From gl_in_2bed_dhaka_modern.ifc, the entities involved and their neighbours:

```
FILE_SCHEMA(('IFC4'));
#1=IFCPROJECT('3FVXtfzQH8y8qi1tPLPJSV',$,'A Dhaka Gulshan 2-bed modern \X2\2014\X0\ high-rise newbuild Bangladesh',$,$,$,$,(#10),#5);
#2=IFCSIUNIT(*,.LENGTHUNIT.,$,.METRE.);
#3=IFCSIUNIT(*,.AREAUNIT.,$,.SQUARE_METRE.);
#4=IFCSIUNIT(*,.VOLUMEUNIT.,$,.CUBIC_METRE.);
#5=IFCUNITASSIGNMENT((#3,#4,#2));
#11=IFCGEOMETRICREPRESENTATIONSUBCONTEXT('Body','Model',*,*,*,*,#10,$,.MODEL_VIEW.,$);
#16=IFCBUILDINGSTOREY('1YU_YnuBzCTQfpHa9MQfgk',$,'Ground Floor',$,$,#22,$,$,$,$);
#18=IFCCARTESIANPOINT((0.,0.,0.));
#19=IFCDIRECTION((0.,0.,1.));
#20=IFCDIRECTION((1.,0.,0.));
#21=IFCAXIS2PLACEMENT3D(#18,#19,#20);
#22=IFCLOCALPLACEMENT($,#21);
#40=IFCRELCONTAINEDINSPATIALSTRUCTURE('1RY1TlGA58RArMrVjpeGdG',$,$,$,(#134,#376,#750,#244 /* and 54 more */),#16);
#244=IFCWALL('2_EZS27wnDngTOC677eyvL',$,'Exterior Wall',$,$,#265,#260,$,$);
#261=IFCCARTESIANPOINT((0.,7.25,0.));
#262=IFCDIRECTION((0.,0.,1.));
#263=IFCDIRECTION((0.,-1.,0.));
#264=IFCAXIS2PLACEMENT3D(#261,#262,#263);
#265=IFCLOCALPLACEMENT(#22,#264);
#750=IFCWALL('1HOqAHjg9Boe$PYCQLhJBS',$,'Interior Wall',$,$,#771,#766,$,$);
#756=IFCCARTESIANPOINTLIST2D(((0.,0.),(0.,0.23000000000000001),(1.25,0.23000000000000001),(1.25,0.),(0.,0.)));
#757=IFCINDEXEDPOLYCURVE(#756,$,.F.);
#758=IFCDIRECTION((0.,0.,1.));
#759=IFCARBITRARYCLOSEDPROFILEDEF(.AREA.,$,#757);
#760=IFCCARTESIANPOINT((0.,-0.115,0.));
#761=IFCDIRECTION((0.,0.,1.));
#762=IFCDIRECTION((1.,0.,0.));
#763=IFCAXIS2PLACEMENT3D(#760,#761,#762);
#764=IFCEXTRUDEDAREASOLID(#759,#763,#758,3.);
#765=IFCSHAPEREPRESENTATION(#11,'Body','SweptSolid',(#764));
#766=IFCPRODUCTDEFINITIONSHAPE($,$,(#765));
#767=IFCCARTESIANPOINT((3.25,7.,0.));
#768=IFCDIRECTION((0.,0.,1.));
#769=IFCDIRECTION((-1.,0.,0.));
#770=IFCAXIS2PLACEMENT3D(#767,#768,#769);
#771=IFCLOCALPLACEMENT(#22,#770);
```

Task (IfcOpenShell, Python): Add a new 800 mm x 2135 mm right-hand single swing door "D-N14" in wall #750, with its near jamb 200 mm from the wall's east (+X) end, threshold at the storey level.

```python
import numpy as np
import ifcopenshell
import ifcopenshell.api.feature
import ifcopenshell.api.geometry
import ifcopenshell.api.root
import ifcopenshell.api.spatial
import ifcopenshell.geom
import ifcopenshell.util.element
import ifcopenshell.util.placement
import ifcopenshell.util.representation
import ifcopenshell.util.shape
import ifcopenshell.util.unit

model = ifcopenshell.open("gl_in_2bed_dhaka_modern.ifc")
unit_scale = ifcopenshell.util.unit.calculate_unit_scale(model)
settings = ifcopenshell.geom.settings()


def volume(element):
    """Net volume in cubic metres, openings subtracted."""
    shape = ifcopenshell.geom.create_shape(settings, element)
    return ifcopenshell.util.shape.get_volume(shape.geometry)


wall = model.by_guid("1HOqAHjg9Boe$PYCQLhJBS")
storey = ifcopenshell.util.element.get_container(wall, ifc_class="IfcBuildingStorey")
context = ifcopenshell.util.representation.get_context(model, "Model", "Body", "MODEL_VIEW")
before = volume(wall)

width, height, from_end, sill = 0.8, 2.135, 0.2, 0.0  # metres

# The wall runs along its own X axis, and the end named is its -X end.
wall_shape = ifcopenshell.geom.create_shape(settings, wall)
x, y, z = ifcopenshell.util.shape.get_vertices(wall_shape.geometry).T
start = x.min() + from_end
face, thickness = float(y.min()), float(y.max() - y.min())
wall_matrix = ifcopenshell.util.placement.get_local_placement(wall.ObjectPlacement)
level = ifcopenshell.util.placement.get_local_placement(storey.ObjectPlacement)[2, 3]


def in_wall(x, y):
    """Placement at x, y metres in the wall's axes, at sill height."""
    matrix = wall_matrix.copy()
    matrix[:, 3] = wall_matrix @ np.array([x / unit_scale, y / unit_scale, 0.0, 1.0])
    matrix[2, 3] = level + sill / unit_scale
    return matrix


# Opening: a box that overshoots both wall faces by 50 mm.
opening = ifcopenshell.api.root.create_entity(model, ifc_class="IfcOpeningElement", predefined_type="OPENING")
box = ifcopenshell.api.geometry.add_wall_representation(
    model, context=context, length=width, height=height, thickness=thickness + 0.1
)
ifcopenshell.api.geometry.assign_representation(model, product=opening, representation=box)
ifcopenshell.api.geometry.edit_object_placement(model, product=opening, matrix=in_wall(start, face - 0.05), is_si=False)
ifcopenshell.api.feature.add_feature(model, feature=opening, element=wall)

door = ifcopenshell.api.root.create_entity(model, ifc_class="IfcDoor", name="D-N14", predefined_type="DOOR")
door.OverallWidth, door.OverallHeight = width / unit_scale, height / unit_scale
door.OperationType = "SINGLE_SWING_RIGHT"
body = ifcopenshell.api.geometry.add_door_representation(
    model,
    context=context,
    overall_width=door.OverallWidth,
    overall_height=door.OverallHeight,
    operation_type="SINGLE_SWING_RIGHT",
    lining_properties={"LiningDepth": thickness / unit_scale, "ThresholdDepth": thickness / unit_scale},
)
ifcopenshell.api.geometry.assign_representation(model, product=door, representation=body)
ifcopenshell.api.spatial.assign_container(model, products=[door], relating_structure=storey)
ifcopenshell.api.feature.add_filling(model, opening=opening, element=door)

# The lining spans the wall, so the door starts at the wall face.
ifcopenshell.api.geometry.edit_object_placement(model, product=door, matrix=in_wall(start, face), is_si=False)

after = volume(wall)

print(f"wall volume {before:.3f} -> {after:.3f} m3")

model.write("gl_in_2bed_dhaka_modern_v2.ifc")
```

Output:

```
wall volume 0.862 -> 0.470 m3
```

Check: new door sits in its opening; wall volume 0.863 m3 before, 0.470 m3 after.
